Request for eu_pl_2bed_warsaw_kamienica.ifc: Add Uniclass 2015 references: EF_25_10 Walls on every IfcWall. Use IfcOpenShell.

First a look at what the model holds.

```python
import ifcopenshell

model = ifcopenshell.open("eu_pl_2bed_warsaw_kamienica.ifc")
print(model.schema)
print("classifications:", [c.Name for c in model.by_type("IfcClassification")])
for ifc_class in ("IfcDoor", "IfcRoof", "IfcStair", "IfcWall", "IfcWindow"):
    print(ifc_class, len(model.by_type(ifc_class)))
```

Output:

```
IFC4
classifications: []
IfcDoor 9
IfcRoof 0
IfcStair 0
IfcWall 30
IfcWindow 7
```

```python
import ifcopenshell
import ifcopenshell.api.classification

model = ifcopenshell.open("eu_pl_2bed_warsaw_kamienica.ifc")

system = ifcopenshell.api.classification.add_classification(model, classification="Uniclass 2015")

codes = {
    "IfcWall": ("EF_25_10", "Walls"),
}
for ifc_class, (code, name) in codes.items():
    products = model.by_type(ifc_class)
    ifcopenshell.api.classification.add_reference(
        model, products=products, classification=system, identification=code, name=name
    )
    print(code, len(products))

model.write("eu_pl_2bed_warsaw_kamienica_updated.ifc")
```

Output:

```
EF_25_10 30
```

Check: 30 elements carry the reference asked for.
